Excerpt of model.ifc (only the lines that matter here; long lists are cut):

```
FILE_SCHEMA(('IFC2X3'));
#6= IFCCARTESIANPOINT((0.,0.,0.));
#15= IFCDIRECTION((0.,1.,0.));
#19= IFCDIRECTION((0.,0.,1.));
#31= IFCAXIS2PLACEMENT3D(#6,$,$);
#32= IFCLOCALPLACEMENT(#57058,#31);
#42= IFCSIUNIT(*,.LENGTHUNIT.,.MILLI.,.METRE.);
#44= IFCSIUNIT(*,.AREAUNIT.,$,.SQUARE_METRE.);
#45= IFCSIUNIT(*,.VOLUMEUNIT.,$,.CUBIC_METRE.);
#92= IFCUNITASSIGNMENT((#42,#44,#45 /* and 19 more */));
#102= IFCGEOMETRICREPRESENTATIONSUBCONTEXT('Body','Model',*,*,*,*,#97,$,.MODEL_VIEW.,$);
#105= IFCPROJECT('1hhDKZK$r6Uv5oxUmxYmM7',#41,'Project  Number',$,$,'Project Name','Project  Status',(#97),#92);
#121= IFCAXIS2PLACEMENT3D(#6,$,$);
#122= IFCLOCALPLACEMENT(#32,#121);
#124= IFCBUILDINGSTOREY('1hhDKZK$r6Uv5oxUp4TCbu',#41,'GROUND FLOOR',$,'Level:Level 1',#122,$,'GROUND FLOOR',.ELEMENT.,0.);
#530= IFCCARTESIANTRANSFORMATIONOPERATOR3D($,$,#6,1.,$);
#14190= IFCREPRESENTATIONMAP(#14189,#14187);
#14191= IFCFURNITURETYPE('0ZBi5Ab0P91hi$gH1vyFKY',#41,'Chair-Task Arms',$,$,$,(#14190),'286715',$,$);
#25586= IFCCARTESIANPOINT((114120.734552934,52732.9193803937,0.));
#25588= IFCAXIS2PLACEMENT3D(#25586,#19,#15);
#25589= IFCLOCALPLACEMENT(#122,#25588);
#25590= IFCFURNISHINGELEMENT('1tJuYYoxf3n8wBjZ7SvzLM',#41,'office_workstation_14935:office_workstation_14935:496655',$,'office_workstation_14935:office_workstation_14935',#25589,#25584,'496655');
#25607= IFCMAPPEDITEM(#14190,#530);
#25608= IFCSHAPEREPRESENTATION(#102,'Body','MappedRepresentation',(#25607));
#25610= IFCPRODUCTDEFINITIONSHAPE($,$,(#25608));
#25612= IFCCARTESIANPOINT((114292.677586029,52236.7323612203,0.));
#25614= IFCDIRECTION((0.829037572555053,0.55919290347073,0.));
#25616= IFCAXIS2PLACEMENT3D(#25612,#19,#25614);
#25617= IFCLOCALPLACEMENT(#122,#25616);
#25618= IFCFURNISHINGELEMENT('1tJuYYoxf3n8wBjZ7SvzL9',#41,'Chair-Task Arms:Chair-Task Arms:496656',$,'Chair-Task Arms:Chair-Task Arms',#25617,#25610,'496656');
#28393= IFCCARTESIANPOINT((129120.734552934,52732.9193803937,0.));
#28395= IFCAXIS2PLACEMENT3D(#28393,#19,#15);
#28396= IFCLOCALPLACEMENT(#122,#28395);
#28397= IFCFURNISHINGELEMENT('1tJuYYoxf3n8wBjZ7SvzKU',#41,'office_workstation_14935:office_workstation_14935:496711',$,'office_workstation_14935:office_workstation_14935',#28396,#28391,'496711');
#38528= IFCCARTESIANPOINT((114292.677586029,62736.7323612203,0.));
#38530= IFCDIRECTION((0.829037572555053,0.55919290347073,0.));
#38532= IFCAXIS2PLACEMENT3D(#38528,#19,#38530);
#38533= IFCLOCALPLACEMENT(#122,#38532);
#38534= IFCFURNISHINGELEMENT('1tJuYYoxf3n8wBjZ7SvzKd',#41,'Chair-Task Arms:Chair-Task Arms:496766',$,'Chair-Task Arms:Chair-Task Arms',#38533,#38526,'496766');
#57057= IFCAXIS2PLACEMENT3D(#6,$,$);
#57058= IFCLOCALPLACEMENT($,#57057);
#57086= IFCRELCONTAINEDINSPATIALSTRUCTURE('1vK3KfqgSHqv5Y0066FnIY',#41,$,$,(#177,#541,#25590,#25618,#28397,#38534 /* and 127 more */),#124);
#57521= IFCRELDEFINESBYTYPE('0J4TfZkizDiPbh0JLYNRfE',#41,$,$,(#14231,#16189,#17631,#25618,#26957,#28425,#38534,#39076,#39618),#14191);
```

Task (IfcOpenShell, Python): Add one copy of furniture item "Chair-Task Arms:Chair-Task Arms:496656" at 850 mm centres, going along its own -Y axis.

```python
import ifcopenshell
import ifcopenshell.api.geometry
import ifcopenshell.api.root
import ifcopenshell.util.element
import ifcopenshell.util.placement
import ifcopenshell.util.unit

model = ifcopenshell.open("model.ifc")
unit_scale = ifcopenshell.util.unit.calculate_unit_scale(model)


def reuse_history(source, copy):
    """copy_class also copies each property set's owner history, people and application; keep the originals."""
    for rel in copy.IsDefinedBy:
        if rel.is_a("IfcRelDefinesByProperties") and (history := rel.RelatingPropertyDefinition.OwnerHistory):
            rel.RelatingPropertyDefinition.OwnerHistory = source.OwnerHistory
            ifcopenshell.util.element.remove_deep2(model, history)


source = model.by_id(25618)
base = ifcopenshell.util.placement.get_local_placement(source.ObjectPlacement)
step = -base[:3, 1] * 0.85 / unit_scale

for i in range(1, 2):
    copy = ifcopenshell.api.root.copy_class(model, product=source)
    copy.Representation = ifcopenshell.util.element.copy_deep(
        model, source.Representation, exclude=["IfcGeometricRepresentationContext", "IfcRepresentationMap"]
    )
    copy.Name = "Chair-Task Arms:Chair-Task Arms"
    copy.Tag = None
    reuse_history(source, copy)
    matrix = base.copy()
    matrix[:3, 3] += i * step
    print("added at", matrix[:3, 3].round(3) + 0.0)
    ifcopenshell.api.geometry.edit_object_placement(model, product=copy, matrix=matrix, is_si=False)

model.write("model_updated.ifc")
```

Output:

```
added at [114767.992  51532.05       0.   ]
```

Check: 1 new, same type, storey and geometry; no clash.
